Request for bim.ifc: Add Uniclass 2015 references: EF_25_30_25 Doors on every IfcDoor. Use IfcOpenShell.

First a look at what the model holds.

```python
import ifcopenshell

model = ifcopenshell.open("bim.ifc")
print(model.schema)
print("classifications:", [c.Name for c in model.by_type("IfcClassification")])
for ifc_class in ("IfcDoor", "IfcRoof", "IfcStair", "IfcWall", "IfcWindow"):
    print(ifc_class, len(model.by_type(ifc_class)))
```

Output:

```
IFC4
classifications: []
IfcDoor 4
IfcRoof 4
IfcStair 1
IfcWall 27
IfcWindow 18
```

```python
import ifcopenshell
import ifcopenshell.api.classification

model = ifcopenshell.open("bim.ifc")

system = ifcopenshell.api.classification.add_classification(model, classification="Uniclass 2015")

codes = {
    "IfcDoor": ("EF_25_30_25", "Doors"),
}
for ifc_class, (code, name) in codes.items():
    products = model.by_type(ifc_class)
    ifcopenshell.api.classification.add_reference(
        model, products=products, classification=system, identification=code, name=name
    )
    print(code, len(products))

model.write("bim_updated.ifc")
```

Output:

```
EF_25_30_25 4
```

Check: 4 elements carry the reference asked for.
